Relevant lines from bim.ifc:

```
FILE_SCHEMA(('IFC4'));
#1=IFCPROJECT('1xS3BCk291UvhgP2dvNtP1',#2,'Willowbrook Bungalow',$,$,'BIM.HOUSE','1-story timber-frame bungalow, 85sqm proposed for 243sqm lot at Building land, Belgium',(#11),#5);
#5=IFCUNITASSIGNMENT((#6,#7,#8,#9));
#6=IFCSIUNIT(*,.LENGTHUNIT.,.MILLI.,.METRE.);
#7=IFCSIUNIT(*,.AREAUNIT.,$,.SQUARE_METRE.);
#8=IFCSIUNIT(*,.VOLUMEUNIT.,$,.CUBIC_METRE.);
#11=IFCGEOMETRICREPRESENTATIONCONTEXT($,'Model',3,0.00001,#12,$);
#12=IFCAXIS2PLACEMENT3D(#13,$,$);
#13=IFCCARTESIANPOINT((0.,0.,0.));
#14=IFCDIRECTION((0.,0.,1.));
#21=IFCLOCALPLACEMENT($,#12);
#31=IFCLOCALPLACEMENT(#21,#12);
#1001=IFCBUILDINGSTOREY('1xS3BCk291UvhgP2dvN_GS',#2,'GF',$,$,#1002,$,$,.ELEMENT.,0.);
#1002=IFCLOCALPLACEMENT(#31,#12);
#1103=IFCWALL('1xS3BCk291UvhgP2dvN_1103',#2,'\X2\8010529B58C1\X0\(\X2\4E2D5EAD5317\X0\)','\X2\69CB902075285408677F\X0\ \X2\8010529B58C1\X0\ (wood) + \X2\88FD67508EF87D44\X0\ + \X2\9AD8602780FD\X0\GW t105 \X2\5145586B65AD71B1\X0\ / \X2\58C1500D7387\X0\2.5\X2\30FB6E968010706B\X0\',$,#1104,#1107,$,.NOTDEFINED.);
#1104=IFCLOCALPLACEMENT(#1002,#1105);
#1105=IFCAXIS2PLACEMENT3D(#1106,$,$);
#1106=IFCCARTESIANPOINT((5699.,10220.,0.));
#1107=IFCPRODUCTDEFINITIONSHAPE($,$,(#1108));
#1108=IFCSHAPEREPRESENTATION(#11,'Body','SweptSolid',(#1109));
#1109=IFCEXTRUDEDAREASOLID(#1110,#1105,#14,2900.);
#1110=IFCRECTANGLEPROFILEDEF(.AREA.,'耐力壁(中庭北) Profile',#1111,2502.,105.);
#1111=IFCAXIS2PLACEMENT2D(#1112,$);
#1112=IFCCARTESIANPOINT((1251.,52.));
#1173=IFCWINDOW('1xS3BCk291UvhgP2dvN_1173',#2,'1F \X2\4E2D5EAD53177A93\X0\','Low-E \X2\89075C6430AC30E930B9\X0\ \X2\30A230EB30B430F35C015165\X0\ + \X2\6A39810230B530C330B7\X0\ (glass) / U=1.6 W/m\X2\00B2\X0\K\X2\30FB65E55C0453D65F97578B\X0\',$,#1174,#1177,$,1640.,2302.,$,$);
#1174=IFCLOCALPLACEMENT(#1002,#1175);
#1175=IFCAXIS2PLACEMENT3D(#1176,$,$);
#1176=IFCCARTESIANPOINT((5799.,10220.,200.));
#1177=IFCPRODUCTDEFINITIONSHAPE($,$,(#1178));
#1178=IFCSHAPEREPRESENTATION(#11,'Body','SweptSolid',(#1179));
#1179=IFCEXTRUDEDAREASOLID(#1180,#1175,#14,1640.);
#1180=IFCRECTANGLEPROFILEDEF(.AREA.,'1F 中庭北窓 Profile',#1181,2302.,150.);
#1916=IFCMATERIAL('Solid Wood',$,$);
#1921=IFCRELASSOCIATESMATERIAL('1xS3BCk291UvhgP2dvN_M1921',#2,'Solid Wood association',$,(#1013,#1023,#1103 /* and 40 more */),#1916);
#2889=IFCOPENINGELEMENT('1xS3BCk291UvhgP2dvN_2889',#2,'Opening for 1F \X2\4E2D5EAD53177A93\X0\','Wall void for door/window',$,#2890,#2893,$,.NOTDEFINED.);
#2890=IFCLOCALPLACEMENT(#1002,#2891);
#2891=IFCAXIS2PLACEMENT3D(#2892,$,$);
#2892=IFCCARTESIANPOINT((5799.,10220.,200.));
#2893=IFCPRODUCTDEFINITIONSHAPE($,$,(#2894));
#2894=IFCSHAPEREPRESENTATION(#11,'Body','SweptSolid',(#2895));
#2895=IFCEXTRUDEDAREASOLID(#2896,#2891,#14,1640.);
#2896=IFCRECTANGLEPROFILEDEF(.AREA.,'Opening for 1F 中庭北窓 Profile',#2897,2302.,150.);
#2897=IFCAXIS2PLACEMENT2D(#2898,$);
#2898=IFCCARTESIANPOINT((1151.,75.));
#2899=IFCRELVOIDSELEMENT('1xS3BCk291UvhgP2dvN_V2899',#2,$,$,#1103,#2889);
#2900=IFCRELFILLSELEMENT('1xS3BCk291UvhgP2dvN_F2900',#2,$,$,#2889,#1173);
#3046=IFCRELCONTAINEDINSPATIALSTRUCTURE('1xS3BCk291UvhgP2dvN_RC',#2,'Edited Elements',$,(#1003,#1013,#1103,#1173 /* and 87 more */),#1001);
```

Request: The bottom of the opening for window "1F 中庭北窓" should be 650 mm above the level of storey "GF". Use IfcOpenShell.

```python
import numpy as np
import ifcopenshell
import ifcopenshell.api.geometry
import ifcopenshell.geom
import ifcopenshell.util.element
import ifcopenshell.util.placement
import ifcopenshell.util.shape
import ifcopenshell.util.unit

model = ifcopenshell.open("bim.ifc")
unit_scale = ifcopenshell.util.unit.calculate_unit_scale(model)

window = model.by_guid("1xS3BCk291UvhgP2dvN_1173")
opening = window.FillsVoids[0].RelatingOpeningElement
storey = ifcopenshell.util.element.get_container(window, ifc_class="IfcBuildingStorey")
level = ifcopenshell.util.placement.get_local_placement(storey.ObjectPlacement)[2, 3]

# The opening's origin need not be at the sill, so measure its lowest point.
shape = ifcopenshell.geom.create_shape(ifcopenshell.geom.settings(), opening)
bottom = ifcopenshell.util.shape.get_shape_bottom_elevation(shape, shape.geometry) / unit_scale
dz = level + 650.0 - bottom

shift = np.array([0.0, 0.0, dz])
# The window is not placed relative to its opening, so move both.
for product in (opening, window):
    matrix = ifcopenshell.util.placement.get_local_placement(product.ObjectPlacement)
    matrix[:3, 3] += shift
    ifcopenshell.api.geometry.edit_object_placement(model, product=product, matrix=matrix, is_si=False)

print(f"moved by {dz * unit_scale:+.3f} m")

model.write("bim-out.ifc")
```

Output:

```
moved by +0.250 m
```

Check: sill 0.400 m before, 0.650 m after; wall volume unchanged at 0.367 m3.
